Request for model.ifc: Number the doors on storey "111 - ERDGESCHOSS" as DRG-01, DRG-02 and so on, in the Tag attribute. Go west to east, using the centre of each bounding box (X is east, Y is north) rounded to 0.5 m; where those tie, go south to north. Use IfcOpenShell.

First a look at what the model holds.

```python
import ifcopenshell
import ifcopenshell.util.element
import ifcopenshell.util.placement

model = ifcopenshell.open("model.ifc")
print(model.schema)
storey = next(s for s in model.by_type("IfcBuildingStorey") if s.Name == "111 - ERDGESCHOSS")
doors = [e for e in ifcopenshell.util.element.get_decomposition(storey) if e.is_a("IfcDoor")]
for e in sorted(doors, key=lambda e: e.id()):
    origin = ifcopenshell.util.placement.get_local_placement(e.ObjectPlacement)[:3, 3]
    print(e.id(), e.Tag, e.Name, origin.round(2) + 0.0, sep=" | ")
```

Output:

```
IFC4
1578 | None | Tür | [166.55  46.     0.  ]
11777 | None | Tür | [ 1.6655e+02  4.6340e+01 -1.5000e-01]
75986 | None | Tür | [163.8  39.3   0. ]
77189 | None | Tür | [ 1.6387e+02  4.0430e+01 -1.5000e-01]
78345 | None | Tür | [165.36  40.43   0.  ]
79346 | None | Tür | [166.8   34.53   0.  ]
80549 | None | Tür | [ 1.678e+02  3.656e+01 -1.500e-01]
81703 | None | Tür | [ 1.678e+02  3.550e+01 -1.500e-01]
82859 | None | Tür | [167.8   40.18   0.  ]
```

```python
import ifcopenshell
import ifcopenshell.geom
import ifcopenshell.util.element
import ifcopenshell.util.shape

model = ifcopenshell.open("model.ifc")
settings = ifcopenshell.geom.settings()
settings.set("use-world-coords", True)


def centre(element):
    shape = ifcopenshell.geom.create_shape(settings, element)
    return ifcopenshell.util.shape.get_bbox_centroid(shape.geometry)


storey = next(s for s in model.by_type("IfcBuildingStorey") if s.Name == "111 - ERDGESCHOSS")
doors = [e for e in ifcopenshell.util.element.get_decomposition(storey) if e.is_a("IfcDoor")]

# Insertion points can sit at a corner or the storey origin, so sort by the geometry (in metres).
centres = {e: centre(e) for e in doors}
doors.sort(key=lambda e: (round(centres[e][0] / 0.5), centres[e][1]))

for i, e in enumerate(doors, start=1):
    number = f"DRG-{i:02d}"
    e.Tag = number
    print(e.id(), number)

model.write("model_edited.ifc")
```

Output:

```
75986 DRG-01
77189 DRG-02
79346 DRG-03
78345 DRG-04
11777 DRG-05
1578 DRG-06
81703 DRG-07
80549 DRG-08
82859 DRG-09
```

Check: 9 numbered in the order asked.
